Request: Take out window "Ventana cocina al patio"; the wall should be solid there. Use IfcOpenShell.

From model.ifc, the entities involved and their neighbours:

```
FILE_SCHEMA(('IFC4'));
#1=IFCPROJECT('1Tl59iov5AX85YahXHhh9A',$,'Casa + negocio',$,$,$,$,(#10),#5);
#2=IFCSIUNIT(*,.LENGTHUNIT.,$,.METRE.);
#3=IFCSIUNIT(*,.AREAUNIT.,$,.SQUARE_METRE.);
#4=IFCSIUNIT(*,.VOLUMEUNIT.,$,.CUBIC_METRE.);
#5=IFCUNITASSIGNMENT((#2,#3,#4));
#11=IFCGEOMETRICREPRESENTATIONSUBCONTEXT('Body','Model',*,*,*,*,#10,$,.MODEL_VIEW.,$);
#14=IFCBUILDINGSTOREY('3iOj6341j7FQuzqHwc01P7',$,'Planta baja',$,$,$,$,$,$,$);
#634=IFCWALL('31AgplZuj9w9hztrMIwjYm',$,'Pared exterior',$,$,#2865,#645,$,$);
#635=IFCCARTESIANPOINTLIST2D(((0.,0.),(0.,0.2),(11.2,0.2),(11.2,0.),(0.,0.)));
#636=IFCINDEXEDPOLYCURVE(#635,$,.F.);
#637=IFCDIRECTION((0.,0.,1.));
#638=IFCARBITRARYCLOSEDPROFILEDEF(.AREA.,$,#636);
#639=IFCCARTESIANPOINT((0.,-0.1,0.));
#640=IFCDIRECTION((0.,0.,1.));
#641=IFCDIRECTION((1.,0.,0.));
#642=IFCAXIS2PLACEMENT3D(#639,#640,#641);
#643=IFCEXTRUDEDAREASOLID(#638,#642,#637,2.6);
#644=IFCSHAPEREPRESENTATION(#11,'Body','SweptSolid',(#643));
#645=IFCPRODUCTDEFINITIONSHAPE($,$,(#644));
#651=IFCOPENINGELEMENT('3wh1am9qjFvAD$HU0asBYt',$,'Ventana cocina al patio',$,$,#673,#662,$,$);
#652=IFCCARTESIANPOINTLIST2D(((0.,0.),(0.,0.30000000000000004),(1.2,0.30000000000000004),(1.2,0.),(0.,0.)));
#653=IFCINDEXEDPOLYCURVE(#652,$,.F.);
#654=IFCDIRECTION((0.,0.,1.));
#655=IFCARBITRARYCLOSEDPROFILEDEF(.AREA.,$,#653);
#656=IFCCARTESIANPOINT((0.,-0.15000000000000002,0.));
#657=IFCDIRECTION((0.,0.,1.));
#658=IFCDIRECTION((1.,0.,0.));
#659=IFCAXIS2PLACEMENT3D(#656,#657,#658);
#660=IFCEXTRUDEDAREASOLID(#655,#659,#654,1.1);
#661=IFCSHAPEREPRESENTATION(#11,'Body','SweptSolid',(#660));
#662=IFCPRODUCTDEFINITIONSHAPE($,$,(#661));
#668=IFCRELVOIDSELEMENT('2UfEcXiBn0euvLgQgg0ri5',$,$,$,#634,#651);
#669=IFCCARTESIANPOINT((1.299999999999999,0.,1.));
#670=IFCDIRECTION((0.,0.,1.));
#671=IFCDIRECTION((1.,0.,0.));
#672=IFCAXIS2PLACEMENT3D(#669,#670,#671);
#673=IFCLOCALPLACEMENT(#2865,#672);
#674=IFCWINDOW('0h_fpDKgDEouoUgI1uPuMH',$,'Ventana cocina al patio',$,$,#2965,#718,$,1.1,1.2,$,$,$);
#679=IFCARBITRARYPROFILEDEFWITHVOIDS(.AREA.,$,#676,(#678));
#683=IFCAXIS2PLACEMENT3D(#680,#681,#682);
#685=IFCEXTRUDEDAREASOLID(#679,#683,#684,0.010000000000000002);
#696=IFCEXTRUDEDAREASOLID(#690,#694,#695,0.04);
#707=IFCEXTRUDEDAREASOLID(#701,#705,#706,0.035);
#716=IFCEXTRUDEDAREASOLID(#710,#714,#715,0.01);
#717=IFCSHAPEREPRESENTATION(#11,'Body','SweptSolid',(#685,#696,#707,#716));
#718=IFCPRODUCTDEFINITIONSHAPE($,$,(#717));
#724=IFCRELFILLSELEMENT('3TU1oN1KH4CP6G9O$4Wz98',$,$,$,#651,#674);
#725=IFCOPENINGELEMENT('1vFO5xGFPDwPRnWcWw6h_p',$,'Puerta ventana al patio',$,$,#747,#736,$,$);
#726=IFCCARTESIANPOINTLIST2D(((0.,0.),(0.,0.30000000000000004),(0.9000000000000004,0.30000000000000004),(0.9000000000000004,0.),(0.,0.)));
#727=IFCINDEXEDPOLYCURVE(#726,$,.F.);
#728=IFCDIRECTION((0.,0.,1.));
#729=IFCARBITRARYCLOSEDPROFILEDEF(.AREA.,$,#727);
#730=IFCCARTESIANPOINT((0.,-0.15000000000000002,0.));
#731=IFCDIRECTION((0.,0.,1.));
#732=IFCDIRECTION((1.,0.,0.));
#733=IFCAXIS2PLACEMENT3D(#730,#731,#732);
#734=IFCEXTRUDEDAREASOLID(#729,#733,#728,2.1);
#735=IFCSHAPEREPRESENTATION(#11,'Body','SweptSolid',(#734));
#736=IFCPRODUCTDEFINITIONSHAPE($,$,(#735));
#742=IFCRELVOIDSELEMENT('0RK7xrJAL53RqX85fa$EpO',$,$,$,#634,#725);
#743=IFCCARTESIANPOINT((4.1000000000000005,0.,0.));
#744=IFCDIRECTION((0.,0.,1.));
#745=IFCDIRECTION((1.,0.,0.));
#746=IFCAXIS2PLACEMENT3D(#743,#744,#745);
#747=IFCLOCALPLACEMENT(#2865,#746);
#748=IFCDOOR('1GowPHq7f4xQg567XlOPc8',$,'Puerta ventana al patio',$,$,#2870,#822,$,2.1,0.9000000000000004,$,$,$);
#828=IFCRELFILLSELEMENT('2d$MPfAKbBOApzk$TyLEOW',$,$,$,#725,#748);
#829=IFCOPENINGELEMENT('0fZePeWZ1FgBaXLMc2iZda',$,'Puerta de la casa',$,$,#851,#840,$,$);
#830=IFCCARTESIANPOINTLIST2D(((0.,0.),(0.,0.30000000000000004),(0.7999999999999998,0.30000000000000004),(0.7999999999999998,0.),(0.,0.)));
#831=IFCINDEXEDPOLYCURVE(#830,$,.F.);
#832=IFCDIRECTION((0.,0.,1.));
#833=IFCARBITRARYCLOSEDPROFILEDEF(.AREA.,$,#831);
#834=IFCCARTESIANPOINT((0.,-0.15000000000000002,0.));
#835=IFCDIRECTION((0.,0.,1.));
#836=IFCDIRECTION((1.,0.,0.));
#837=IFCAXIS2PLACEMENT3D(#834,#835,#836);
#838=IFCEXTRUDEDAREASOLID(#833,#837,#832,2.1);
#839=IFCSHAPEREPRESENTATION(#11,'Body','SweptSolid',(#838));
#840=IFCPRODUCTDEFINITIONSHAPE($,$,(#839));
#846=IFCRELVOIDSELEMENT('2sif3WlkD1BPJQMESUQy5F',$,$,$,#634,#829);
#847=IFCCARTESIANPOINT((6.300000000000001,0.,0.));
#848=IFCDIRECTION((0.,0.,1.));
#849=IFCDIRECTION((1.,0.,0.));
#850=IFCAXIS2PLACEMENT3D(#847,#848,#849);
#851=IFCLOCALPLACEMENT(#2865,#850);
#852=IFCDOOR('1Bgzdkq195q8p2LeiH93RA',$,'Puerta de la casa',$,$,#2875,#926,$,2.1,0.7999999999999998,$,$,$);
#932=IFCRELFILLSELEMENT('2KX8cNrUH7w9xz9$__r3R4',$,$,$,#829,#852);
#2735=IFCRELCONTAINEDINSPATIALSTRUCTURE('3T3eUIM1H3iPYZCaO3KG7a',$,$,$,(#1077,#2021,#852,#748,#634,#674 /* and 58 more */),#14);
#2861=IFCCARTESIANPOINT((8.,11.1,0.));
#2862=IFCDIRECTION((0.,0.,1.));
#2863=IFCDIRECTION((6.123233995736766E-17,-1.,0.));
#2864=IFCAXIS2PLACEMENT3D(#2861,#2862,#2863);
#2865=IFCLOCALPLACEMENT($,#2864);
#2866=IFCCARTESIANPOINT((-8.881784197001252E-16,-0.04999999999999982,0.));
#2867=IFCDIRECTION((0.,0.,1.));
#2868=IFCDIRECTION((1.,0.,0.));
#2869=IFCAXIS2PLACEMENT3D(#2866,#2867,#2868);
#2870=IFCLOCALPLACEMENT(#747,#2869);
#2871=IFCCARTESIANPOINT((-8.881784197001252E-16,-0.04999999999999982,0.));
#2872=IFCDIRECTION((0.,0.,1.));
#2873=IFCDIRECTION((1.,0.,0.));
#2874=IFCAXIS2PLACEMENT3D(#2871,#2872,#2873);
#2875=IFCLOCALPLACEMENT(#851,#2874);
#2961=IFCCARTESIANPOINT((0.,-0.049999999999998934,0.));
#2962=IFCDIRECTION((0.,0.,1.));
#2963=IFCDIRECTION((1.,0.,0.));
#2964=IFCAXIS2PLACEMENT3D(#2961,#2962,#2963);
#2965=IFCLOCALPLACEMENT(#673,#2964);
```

```python
import ifcopenshell
import ifcopenshell.api.feature
import ifcopenshell.api.root
import ifcopenshell.geom
import ifcopenshell.util.shape

model = ifcopenshell.open("model.ifc")
settings = ifcopenshell.geom.settings()


def volume(element):
    """Net volume in cubic metres, openings subtracted."""
    shape = ifcopenshell.geom.create_shape(settings, element)
    return ifcopenshell.util.shape.get_volume(shape.geometry)


window = model.by_id(674)
opening = window.FillsVoids[0].RelatingOpeningElement
wall = opening.VoidsElements[0].RelatingBuildingElement
before = volume(wall)

ifcopenshell.api.root.remove_product(model, product=window)
ifcopenshell.api.feature.remove_feature(model, feature=opening)

after = volume(wall)

print(f"wall volume {before:.3f} -> {after:.3f} m3")

model.write("model_v2.ifc")
```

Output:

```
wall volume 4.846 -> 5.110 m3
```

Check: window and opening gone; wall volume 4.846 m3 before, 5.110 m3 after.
